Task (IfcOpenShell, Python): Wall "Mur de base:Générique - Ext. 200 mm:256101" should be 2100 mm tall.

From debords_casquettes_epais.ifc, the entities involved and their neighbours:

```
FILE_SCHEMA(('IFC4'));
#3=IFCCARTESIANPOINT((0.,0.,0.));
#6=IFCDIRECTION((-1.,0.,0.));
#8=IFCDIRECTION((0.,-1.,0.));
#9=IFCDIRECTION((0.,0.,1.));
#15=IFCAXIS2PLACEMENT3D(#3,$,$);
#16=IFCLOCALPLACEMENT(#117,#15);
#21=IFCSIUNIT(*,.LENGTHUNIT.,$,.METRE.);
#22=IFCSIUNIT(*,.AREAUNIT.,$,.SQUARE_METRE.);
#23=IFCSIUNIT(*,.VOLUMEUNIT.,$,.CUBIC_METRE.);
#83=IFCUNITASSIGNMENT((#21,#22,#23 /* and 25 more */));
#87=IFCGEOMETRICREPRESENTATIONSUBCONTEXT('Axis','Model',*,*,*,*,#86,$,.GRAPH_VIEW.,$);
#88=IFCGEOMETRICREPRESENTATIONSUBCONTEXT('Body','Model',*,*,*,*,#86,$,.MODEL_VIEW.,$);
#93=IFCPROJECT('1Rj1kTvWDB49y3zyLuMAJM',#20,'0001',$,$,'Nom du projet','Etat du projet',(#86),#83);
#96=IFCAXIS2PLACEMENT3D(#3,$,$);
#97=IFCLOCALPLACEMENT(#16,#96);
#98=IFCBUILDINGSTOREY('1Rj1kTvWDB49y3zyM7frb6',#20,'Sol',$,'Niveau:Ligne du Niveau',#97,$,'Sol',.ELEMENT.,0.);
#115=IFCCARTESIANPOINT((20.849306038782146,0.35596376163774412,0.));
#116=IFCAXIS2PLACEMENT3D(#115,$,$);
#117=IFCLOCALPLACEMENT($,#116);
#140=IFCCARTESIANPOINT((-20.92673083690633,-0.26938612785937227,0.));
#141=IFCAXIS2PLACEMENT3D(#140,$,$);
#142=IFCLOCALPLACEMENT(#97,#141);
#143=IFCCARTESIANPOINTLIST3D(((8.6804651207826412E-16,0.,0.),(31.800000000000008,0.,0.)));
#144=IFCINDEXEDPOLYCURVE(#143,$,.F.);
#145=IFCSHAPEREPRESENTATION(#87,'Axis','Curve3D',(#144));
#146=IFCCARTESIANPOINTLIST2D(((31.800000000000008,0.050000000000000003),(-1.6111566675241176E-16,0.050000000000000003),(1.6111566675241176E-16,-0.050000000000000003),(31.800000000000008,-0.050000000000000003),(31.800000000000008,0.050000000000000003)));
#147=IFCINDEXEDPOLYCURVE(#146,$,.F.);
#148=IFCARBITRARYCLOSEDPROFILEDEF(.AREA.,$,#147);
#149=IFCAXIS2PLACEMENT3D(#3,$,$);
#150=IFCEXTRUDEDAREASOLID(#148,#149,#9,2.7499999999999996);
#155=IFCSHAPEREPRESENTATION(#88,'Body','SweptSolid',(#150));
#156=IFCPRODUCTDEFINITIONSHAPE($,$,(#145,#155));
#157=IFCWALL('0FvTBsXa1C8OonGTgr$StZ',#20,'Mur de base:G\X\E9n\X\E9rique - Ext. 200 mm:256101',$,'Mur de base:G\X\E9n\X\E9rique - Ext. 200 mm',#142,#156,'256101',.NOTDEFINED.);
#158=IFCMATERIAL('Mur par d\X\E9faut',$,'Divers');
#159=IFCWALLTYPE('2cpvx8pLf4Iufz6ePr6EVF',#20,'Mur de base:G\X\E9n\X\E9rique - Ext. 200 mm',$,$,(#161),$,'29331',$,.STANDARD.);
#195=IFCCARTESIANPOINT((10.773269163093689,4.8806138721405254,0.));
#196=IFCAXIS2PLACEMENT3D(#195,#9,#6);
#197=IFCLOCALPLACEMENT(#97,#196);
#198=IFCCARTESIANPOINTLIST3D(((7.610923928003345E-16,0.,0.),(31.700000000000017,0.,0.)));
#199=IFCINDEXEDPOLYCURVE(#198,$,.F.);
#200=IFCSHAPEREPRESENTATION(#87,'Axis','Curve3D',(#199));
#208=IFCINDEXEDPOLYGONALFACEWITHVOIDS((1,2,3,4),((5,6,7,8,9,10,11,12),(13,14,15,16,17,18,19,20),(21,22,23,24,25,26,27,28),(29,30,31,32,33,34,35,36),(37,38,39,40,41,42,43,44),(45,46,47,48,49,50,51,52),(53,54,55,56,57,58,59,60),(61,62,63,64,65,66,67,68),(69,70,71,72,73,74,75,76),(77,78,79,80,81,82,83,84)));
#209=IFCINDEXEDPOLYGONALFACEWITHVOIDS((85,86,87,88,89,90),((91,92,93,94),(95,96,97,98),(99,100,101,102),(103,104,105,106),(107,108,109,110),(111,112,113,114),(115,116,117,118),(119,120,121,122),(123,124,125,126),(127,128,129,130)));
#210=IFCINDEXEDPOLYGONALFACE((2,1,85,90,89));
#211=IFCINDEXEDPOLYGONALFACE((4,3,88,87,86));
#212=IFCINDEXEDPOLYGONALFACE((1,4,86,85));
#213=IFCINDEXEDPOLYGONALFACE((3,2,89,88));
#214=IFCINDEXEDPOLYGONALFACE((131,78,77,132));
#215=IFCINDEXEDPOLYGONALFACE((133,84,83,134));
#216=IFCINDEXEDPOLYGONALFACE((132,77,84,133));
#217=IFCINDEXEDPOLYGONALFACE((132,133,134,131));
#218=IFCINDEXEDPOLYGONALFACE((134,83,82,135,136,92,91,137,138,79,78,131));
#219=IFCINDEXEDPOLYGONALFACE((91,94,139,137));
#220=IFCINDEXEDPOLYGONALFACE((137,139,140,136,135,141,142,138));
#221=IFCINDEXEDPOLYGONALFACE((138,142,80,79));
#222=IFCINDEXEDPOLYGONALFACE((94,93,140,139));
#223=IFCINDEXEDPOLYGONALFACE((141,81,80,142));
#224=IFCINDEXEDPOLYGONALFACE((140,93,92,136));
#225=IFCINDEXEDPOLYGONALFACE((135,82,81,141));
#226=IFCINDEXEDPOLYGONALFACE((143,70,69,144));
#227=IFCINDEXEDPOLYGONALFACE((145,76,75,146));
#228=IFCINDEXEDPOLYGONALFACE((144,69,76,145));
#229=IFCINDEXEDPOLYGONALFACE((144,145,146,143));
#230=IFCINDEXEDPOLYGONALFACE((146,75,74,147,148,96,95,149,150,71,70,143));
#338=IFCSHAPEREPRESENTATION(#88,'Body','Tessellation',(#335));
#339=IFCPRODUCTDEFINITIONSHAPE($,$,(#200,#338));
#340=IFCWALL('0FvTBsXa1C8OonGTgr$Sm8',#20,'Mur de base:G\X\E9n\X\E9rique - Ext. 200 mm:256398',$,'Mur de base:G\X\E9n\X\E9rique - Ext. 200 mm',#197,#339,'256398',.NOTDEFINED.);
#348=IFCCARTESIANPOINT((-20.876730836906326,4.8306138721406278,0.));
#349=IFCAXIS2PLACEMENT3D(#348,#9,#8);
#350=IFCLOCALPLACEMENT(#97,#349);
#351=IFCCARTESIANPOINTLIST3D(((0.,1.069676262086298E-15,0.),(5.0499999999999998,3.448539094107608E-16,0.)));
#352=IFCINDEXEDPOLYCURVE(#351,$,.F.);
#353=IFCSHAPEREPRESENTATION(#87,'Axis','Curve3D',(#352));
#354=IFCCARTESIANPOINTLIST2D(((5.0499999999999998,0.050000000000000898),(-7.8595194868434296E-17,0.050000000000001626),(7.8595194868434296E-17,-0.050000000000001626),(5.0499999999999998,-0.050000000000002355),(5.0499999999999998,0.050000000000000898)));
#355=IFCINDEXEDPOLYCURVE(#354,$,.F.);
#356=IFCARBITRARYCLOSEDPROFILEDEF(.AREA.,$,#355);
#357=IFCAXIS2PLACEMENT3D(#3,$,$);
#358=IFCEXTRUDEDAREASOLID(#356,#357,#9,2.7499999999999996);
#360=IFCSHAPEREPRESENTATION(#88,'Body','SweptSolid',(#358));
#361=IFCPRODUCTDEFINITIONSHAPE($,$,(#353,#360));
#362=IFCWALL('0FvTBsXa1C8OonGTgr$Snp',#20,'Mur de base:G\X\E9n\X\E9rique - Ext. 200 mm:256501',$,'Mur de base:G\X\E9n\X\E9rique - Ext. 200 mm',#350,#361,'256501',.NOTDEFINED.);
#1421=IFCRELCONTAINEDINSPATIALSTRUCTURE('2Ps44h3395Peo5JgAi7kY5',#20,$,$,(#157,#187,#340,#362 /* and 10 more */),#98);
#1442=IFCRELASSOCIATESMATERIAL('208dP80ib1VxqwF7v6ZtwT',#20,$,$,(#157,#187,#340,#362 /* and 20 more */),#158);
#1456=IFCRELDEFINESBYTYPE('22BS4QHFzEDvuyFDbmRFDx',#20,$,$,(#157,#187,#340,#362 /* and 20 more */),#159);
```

```python
import ifcopenshell
import ifcopenshell.geom
import ifcopenshell.util.representation
import ifcopenshell.util.shape
import ifcopenshell.util.unit

model = ifcopenshell.open("debords_casquettes_epais.ifc")
unit_scale = ifcopenshell.util.unit.calculate_unit_scale(model)
settings = ifcopenshell.geom.settings()


def volume(element):
    """Net volume in cubic metres, openings subtracted."""
    shape = ifcopenshell.geom.create_shape(settings, element)
    return ifcopenshell.util.shape.get_volume(shape.geometry)


wall = model.by_id(157)
before = volume(wall)

body = ifcopenshell.util.representation.get_representation(wall, "Model", "Body")
solid = body.Items[0]
old_height = solid.Depth
solid.Depth = 2.1 / unit_scale
after = volume(wall)

print(f"height {old_height:g} -> {solid.Depth:g}, volume {before:.3f} -> {after:.3f} m3")

model.write("debords_casquettes_epais_updated.ifc")
```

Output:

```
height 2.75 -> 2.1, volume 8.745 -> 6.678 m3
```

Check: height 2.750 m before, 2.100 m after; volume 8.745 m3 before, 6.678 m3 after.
